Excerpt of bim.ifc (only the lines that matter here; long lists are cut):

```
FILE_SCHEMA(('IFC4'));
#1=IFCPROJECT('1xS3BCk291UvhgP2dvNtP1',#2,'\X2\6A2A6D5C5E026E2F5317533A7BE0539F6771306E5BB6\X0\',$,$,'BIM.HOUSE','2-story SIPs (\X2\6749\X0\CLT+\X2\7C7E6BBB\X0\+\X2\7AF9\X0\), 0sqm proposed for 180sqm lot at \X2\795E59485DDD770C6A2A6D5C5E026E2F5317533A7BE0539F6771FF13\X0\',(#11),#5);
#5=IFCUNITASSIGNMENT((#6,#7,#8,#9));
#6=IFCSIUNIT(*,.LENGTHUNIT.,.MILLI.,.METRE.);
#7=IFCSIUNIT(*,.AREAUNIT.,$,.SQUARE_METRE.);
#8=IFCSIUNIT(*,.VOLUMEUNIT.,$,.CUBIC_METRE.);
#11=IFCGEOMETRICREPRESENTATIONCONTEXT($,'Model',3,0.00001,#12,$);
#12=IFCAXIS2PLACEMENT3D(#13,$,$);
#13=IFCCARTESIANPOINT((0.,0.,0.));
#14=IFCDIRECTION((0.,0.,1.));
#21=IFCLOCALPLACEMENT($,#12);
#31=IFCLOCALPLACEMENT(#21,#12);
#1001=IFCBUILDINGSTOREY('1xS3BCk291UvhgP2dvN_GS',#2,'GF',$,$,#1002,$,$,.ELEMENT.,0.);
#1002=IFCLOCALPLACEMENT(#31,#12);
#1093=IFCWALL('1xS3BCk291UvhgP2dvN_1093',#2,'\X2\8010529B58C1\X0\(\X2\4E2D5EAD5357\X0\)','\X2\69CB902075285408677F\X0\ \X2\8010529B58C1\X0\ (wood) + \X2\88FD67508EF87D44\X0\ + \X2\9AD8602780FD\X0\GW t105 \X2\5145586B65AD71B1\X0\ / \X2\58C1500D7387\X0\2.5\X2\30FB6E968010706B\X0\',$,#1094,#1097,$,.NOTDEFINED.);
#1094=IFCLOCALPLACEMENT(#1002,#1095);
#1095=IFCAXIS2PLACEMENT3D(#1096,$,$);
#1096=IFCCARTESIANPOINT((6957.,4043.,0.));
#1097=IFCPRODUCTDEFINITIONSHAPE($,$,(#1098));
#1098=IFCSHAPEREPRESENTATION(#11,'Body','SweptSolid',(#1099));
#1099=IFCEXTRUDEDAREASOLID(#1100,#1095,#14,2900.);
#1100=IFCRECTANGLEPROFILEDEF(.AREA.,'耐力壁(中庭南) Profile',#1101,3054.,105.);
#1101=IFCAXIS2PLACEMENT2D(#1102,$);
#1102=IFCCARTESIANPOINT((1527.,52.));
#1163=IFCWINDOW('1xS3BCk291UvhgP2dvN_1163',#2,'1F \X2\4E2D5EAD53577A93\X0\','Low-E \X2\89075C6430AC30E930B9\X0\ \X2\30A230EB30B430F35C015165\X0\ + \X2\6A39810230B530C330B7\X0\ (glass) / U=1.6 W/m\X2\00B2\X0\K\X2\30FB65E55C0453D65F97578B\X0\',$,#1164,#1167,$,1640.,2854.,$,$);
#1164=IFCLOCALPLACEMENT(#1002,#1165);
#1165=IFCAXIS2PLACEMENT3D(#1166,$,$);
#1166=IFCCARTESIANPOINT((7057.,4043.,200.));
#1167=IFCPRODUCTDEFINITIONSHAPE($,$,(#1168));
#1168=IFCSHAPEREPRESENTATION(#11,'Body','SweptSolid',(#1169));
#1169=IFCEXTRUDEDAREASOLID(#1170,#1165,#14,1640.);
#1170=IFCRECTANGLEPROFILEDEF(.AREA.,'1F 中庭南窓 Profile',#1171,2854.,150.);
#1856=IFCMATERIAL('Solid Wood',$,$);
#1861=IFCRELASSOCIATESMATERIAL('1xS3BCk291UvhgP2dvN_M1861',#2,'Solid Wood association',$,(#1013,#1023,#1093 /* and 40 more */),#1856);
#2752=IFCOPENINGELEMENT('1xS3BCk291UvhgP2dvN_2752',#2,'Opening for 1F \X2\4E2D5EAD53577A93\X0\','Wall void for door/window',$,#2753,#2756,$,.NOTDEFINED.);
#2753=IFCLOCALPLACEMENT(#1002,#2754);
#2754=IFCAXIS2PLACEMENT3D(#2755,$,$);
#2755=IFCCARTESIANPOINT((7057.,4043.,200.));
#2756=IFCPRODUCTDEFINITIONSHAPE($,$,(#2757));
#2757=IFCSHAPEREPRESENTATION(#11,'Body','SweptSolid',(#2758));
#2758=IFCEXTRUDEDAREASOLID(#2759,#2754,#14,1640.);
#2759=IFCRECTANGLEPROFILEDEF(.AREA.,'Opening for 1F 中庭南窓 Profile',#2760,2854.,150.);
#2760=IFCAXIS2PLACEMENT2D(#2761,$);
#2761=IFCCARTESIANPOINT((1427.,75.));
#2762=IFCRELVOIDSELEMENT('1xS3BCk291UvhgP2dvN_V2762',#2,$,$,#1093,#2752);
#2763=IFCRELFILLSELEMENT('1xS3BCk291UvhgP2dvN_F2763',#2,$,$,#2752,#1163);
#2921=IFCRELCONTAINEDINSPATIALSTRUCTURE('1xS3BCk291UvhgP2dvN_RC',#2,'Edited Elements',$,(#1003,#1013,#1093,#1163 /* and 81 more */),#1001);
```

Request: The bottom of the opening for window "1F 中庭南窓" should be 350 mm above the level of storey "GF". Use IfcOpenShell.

```python
import numpy as np
import ifcopenshell
import ifcopenshell.api.geometry
import ifcopenshell.geom
import ifcopenshell.util.element
import ifcopenshell.util.placement
import ifcopenshell.util.shape
import ifcopenshell.util.unit

model = ifcopenshell.open("bim.ifc")
unit_scale = ifcopenshell.util.unit.calculate_unit_scale(model)

window = model.by_guid("1xS3BCk291UvhgP2dvN_1163")
opening = window.FillsVoids[0].RelatingOpeningElement
storey = ifcopenshell.util.element.get_container(window, ifc_class="IfcBuildingStorey")
level = ifcopenshell.util.placement.get_local_placement(storey.ObjectPlacement)[2, 3]

# The opening's origin need not be at the sill, so measure its lowest point.
shape = ifcopenshell.geom.create_shape(ifcopenshell.geom.settings(), opening)
bottom = ifcopenshell.util.shape.get_shape_bottom_elevation(shape, shape.geometry) / unit_scale
dz = level + 0.35 / unit_scale - bottom

shift = np.array([0.0, 0.0, dz])
# The window is not placed relative to its opening, so move both.
for product in (opening, window):
    matrix = ifcopenshell.util.placement.get_local_placement(product.ObjectPlacement)
    matrix[:3, 3] += shift
    ifcopenshell.api.geometry.edit_object_placement(model, product=product, matrix=matrix, is_si=False)

print(f"moved by {dz * unit_scale:+.3f} m")

model.write("bim_edited.ifc")
```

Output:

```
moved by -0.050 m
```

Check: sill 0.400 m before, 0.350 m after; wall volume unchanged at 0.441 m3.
